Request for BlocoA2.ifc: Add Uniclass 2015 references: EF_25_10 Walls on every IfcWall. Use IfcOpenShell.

First a look at what the model holds.

```python
import ifcopenshell

model = ifcopenshell.open("BlocoA2.ifc")
print(model.schema)
print("classifications:", [c.Name for c in model.by_type("IfcClassification")])
for ifc_class in ("IfcDoor", "IfcRoof", "IfcStair", "IfcWall", "IfcWindow"):
    print(ifc_class, len(model.by_type(ifc_class)))
```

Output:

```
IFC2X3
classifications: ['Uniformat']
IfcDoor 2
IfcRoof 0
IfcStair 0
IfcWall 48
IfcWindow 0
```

```python
import ifcopenshell
import ifcopenshell.api.classification

model = ifcopenshell.open("BlocoA2.ifc")

# IFC2X3 requires Source and Edition and has no link from the project to the system.
system = model.create_entity("IfcClassification", Source="NBS", Edition="2015", Name="Uniclass 2015")

codes = {
    "IfcWall": ("EF_25_10", "Walls"),
}
for ifc_class, (code, name) in codes.items():
    products = model.by_type(ifc_class)
    ifcopenshell.api.classification.add_reference(
        model, products=products, classification=system, identification=code, name=name
    )
    print(code, len(products))

model.write("BlocoA2_rev.ifc")
```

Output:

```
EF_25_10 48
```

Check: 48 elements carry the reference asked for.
